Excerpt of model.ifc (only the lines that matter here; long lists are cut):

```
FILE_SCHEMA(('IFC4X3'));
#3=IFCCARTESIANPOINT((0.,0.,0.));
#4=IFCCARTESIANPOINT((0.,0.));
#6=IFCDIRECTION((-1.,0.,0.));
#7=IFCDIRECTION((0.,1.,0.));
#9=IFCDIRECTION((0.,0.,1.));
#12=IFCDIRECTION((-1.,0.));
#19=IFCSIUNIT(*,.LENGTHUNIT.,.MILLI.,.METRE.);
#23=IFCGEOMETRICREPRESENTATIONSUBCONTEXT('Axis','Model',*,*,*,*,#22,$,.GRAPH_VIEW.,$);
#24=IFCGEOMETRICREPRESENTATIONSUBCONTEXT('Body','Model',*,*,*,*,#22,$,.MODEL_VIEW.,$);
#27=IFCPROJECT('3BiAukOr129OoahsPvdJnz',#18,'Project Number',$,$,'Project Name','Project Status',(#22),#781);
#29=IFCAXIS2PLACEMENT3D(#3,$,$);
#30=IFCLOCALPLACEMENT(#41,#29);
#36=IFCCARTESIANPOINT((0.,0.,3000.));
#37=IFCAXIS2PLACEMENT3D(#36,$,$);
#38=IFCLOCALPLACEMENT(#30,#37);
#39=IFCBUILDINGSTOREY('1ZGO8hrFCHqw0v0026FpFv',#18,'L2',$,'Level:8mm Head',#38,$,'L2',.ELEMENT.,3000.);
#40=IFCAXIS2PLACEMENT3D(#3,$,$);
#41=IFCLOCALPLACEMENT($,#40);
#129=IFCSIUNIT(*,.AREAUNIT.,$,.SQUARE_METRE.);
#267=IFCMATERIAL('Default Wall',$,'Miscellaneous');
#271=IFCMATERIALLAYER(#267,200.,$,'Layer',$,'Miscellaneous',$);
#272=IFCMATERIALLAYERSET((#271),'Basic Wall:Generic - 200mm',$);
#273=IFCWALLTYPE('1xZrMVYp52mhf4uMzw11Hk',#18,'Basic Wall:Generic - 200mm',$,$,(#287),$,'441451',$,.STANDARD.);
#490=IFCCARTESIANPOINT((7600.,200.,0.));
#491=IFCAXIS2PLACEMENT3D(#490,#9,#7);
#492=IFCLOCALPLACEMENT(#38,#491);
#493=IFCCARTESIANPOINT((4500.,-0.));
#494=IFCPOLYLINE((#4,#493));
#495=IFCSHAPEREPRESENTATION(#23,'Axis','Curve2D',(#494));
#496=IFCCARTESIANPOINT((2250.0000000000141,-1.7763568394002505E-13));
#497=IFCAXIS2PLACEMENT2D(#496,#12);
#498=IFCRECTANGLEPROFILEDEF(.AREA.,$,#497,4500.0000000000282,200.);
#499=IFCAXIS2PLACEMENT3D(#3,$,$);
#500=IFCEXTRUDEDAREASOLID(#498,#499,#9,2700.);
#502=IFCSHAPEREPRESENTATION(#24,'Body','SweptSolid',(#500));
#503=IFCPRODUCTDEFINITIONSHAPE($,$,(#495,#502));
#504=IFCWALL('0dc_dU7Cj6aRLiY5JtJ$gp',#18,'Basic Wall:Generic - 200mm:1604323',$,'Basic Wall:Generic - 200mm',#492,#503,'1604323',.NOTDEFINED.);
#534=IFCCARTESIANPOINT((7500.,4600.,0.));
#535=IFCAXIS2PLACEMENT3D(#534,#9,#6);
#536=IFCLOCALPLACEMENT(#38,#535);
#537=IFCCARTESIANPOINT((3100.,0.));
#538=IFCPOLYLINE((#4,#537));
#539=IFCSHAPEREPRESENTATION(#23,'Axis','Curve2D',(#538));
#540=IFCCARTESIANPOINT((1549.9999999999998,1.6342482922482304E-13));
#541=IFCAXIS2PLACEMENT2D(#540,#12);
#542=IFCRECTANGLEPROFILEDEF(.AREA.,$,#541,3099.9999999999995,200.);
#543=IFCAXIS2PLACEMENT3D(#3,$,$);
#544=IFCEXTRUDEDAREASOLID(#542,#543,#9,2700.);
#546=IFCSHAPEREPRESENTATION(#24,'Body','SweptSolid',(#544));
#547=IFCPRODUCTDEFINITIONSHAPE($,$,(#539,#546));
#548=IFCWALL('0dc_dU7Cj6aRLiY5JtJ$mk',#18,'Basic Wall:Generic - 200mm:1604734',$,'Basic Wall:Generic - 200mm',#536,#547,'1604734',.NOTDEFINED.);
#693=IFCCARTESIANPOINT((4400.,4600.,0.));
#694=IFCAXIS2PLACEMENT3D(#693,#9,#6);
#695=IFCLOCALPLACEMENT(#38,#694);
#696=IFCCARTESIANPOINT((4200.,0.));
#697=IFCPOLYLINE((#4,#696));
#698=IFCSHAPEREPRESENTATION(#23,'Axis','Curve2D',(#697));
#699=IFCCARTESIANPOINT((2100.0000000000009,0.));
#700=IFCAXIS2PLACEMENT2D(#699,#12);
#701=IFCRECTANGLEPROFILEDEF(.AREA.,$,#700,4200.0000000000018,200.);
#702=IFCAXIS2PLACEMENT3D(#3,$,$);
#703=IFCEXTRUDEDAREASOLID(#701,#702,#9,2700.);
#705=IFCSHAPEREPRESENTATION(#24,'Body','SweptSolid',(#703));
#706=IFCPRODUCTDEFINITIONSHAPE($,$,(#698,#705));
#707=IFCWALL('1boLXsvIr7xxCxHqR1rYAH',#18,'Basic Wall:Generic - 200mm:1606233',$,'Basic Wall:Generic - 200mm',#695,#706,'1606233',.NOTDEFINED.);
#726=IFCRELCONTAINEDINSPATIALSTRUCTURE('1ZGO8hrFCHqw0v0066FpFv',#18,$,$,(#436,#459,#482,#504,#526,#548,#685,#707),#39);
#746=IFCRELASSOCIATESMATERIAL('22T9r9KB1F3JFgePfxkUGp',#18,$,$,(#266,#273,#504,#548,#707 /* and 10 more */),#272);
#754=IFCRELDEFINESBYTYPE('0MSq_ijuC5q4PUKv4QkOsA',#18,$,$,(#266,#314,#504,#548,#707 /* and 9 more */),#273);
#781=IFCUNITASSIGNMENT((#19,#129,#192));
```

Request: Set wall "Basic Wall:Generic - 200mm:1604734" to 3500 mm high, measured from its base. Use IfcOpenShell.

```python
import ifcopenshell
import ifcopenshell.geom
import ifcopenshell.util.representation
import ifcopenshell.util.shape

model = ifcopenshell.open("model.ifc")
settings = ifcopenshell.geom.settings()


def volume(element):
    """Net volume in cubic metres, openings subtracted."""
    shape = ifcopenshell.geom.create_shape(settings, element)
    return ifcopenshell.util.shape.get_volume(shape.geometry)


wall = model.by_guid("0dc_dU7Cj6aRLiY5JtJ$mk")
before = volume(wall)

body = ifcopenshell.util.representation.get_representation(wall, "Model", "Body")
solid = body.Items[0]
old_height = solid.Depth
solid.Depth = 3500.0
after = volume(wall)

print(f"height {old_height:g} -> {solid.Depth:g}, volume {before:.3f} -> {after:.3f} m3")

model.write("model-out.ifc")
```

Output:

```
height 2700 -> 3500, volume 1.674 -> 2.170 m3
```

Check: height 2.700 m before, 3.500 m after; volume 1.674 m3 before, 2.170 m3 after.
